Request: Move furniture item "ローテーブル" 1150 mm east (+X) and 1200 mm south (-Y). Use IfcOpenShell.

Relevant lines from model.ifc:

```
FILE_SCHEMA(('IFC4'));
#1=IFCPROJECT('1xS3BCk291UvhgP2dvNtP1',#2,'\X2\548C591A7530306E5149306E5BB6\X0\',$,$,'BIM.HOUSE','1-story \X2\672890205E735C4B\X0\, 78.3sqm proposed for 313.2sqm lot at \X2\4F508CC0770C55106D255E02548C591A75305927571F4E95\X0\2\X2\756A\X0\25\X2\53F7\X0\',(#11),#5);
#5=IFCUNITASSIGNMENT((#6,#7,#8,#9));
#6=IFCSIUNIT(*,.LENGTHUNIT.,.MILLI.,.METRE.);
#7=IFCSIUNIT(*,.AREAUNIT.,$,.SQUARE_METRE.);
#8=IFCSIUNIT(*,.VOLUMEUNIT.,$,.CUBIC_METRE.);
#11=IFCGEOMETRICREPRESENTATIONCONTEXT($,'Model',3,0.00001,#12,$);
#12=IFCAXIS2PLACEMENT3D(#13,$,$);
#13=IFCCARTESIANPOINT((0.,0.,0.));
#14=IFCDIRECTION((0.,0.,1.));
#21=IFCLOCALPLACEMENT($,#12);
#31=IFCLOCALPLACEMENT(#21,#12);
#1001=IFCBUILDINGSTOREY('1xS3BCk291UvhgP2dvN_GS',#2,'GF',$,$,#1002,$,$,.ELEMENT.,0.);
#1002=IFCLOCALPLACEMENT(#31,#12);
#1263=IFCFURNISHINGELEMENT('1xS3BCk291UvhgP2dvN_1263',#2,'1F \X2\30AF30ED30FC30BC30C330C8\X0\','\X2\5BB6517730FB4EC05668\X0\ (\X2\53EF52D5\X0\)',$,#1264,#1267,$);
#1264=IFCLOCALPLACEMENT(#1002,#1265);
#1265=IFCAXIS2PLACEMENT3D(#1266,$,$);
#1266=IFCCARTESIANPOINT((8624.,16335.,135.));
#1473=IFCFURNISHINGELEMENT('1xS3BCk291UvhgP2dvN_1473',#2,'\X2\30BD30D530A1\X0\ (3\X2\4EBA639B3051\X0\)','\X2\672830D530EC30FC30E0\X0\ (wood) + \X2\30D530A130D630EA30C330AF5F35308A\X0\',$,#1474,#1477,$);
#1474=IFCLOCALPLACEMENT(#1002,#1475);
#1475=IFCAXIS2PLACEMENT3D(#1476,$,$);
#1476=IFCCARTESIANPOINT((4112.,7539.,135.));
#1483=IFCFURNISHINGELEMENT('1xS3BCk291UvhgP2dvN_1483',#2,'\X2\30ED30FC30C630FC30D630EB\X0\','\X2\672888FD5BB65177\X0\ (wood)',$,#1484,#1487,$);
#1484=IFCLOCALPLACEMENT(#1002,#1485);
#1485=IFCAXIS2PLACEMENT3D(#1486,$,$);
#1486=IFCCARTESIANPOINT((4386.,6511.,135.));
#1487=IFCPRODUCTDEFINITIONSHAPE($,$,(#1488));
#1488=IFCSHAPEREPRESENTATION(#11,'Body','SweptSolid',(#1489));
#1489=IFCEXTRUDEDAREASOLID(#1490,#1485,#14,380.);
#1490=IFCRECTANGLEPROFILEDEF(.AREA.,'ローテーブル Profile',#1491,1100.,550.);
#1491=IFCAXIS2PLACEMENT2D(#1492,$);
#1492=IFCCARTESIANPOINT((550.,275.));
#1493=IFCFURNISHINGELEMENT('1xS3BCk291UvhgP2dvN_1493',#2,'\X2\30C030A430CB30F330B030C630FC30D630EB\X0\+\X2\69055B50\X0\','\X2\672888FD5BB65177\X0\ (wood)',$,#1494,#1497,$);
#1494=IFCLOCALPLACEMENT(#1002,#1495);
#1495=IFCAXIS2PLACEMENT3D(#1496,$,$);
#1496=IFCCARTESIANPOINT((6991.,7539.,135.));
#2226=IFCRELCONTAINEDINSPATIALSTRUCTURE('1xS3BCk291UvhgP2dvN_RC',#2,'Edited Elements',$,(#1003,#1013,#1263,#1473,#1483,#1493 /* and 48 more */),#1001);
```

```python
import ifcopenshell
import ifcopenshell.api.geometry
import ifcopenshell.util.placement

model = ifcopenshell.open("model.ifc")

item = model.by_guid("1xS3BCk291UvhgP2dvN_1483")
matrix = ifcopenshell.util.placement.get_local_placement(item.ObjectPlacement)
matrix[0, 3] += 1150.0
matrix[1, 3] -= 1200.0
ifcopenshell.api.geometry.edit_object_placement(model, product=item, matrix=matrix, is_si=False)

print(ifcopenshell.util.placement.get_local_placement(item.ObjectPlacement).round(3) + 0.0)

model.write("model_rev.ifc")
```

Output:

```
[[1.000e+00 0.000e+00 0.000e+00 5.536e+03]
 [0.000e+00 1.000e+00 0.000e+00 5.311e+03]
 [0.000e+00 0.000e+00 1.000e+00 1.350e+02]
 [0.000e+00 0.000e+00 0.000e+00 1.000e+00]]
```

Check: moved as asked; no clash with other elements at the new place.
